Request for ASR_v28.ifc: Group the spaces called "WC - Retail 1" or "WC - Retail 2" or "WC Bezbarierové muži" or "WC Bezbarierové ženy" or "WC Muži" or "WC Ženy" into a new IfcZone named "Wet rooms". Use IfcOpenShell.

First a look at what the model holds.

```python
import ifcopenshell

model = ifcopenshell.open("ASR_v28.ifc")
print(model.schema)
seen = {}
for space in model.by_type("IfcSpace"):
    seen[space.LongName] = seen.get(space.LongName, 0) + 1
for name, count in sorted(seen.items(), key=str):
    print(count, "x", name)
print("zones:", [z.Name for z in model.by_type("IfcZone")][:20])
```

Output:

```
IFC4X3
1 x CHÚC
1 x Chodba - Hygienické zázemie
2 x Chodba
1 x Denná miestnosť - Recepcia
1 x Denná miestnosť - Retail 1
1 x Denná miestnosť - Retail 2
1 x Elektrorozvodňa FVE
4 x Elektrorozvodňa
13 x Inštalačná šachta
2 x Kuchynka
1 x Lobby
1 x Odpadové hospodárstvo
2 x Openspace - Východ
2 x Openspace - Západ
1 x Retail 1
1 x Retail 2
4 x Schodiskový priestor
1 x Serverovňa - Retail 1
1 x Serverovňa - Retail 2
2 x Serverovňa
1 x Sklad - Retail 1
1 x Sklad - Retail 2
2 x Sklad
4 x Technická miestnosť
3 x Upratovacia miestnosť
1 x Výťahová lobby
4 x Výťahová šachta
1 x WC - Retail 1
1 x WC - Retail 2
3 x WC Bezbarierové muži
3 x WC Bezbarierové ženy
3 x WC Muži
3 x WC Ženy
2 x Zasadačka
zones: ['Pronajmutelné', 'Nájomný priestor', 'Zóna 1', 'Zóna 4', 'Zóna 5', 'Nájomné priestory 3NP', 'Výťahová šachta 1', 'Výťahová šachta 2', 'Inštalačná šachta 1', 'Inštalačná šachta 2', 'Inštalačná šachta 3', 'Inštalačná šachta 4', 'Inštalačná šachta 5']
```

```python
import ifcopenshell
import ifcopenshell.api.group
import ifcopenshell.api.root

model = ifcopenshell.open("ASR_v28.ifc")

names = {"WC - Retail 1", "WC - Retail 2", "WC Bezbarierové muži", "WC Bezbarierové ženy", "WC Muži", "WC Ženy"}
spaces = [s for s in model.by_type("IfcSpace") if s.LongName in names]

zone = ifcopenshell.api.root.create_entity(model, ifc_class="IfcZone", name="Wet rooms")
ifcopenshell.api.group.assign_group(model, products=spaces, group=zone)
print(len(spaces), "spaces in", zone.Name)

model.write("ASR_v28_edited.ifc")
```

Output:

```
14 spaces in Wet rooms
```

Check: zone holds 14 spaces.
